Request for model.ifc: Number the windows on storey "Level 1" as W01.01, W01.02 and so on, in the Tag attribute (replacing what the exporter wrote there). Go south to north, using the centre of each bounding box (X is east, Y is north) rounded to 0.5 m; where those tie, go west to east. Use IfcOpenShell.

First a look at what the model holds.

```python
import ifcopenshell
import ifcopenshell.util.element
import ifcopenshell.util.placement

model = ifcopenshell.open("model.ifc")
print(model.schema)
storey = next(s for s in model.by_type("IfcBuildingStorey") if s.Name == "Level 1")
windows = [e for e in ifcopenshell.util.element.get_decomposition(storey) if e.is_a("IfcWindow")]
for e in sorted(windows, key=lambda e: e.id()):
    origin = ifcopenshell.util.placement.get_local_placement(e.ObjectPlacement)[:3, 3]
    print(e.id(), e.Tag, e.Name, origin.round(2) + 0.0, sep=" | ")
```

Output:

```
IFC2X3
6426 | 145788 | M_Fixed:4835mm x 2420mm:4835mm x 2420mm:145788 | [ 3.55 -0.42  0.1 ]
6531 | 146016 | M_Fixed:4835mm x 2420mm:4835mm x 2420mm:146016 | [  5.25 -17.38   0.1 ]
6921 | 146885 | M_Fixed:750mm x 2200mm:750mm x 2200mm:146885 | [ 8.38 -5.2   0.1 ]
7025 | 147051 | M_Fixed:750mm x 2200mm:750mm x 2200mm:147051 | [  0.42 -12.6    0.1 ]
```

```python
import ifcopenshell
import ifcopenshell.geom
import ifcopenshell.util.element
import ifcopenshell.util.shape

model = ifcopenshell.open("model.ifc")
settings = ifcopenshell.geom.settings()
settings.set("use-world-coords", True)


def centre(element):
    shape = ifcopenshell.geom.create_shape(settings, element)
    return ifcopenshell.util.shape.get_bbox_centroid(shape.geometry)


storey = next(s for s in model.by_type("IfcBuildingStorey") if s.Name == "Level 1")
windows = [e for e in ifcopenshell.util.element.get_decomposition(storey) if e.is_a("IfcWindow")]

# Insertion points can sit at a corner or the storey origin, so sort by the geometry (in metres).
centres = {e: centre(e) for e in windows}
windows.sort(key=lambda e: (round(centres[e][1] / 0.5), centres[e][0]))

for i, e in enumerate(windows, start=1):
    number = f"W01.{i:02d}"
    e.Tag = number
    print(e.id(), number)

model.write("model_rev.ifc")
```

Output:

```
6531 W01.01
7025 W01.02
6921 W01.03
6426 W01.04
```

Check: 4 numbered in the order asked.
